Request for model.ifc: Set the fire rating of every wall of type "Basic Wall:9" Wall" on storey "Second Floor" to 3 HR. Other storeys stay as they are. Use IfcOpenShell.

First a look at what the model holds.

```python
import ifcopenshell
import ifcopenshell.util.element

model = ifcopenshell.open("model.ifc")
print(model.schema)
storey = next(s for s in model.by_type("IfcBuildingStorey") if s.Name == "Second Floor")
walls = [e for e in ifcopenshell.util.element.get_decomposition(storey) if e.is_a("IfcWall")]
seen = {}
for e in walls:
    element_type = ifcopenshell.util.element.get_type(e)
    key = (element_type.Name if element_type != e and element_type else None, ifcopenshell.util.element.get_pset(e, "Pset_WallCommon", "FireRating"))
    seen[key] = seen.get(key, 0) + 1
for (name, value), count in sorted(seen.items(), key=str):
    print(count, "x", name, "|", value)
```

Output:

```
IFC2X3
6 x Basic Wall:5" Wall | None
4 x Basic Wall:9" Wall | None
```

```python
import ifcopenshell
import ifcopenshell.api.pset
import ifcopenshell.util.element

model = ifcopenshell.open("model.ifc")

storey = next(s for s in model.by_type("IfcBuildingStorey") if s.Name == "Second Floor")
walls = [e for e in ifcopenshell.util.element.get_decomposition(storey) if e.is_a("IfcWall")]

count = 0
for e in walls:
    element_type = ifcopenshell.util.element.get_type(e)
    if element_type in (None, e) or element_type.Name != 'Basic Wall:9" Wall':
        continue
    # add_pset returns the element's existing set when there is one.
    pset = ifcopenshell.api.pset.add_pset(model, product=e, name="Pset_WallCommon")
    ifcopenshell.api.pset.edit_pset(model, pset=pset, properties={"FireRating": "3 HR"})
    count += 1

print(count, "walls updated")

model.write("model_rev.ifc")
```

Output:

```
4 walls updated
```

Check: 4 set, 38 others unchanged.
